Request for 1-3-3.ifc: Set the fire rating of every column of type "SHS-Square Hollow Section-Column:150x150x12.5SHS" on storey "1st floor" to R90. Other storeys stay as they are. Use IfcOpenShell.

First a look at what the model holds.

```python
import ifcopenshell
import ifcopenshell.util.element

model = ifcopenshell.open("1-3-3.ifc")
print(model.schema)
storey = next(s for s in model.by_type("IfcBuildingStorey") if s.Name == "1st floor")
columns = [e for e in ifcopenshell.util.element.get_decomposition(storey) if e.is_a("IfcColumn")]
seen = {}
for e in columns:
    element_type = ifcopenshell.util.element.get_type(e)
    key = (element_type.Name if element_type != e and element_type else None, ifcopenshell.util.element.get_pset(e, "Pset_ColumnCommon", "FireRating"))
    seen[key] = seen.get(key, 0) + 1
for (name, value), count in sorted(seen.items(), key=str):
    print(count, "x", name, "|", value)
```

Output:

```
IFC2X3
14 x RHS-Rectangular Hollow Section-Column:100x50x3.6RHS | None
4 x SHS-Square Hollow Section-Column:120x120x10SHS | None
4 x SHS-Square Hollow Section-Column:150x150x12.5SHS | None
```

```python
import ifcopenshell
import ifcopenshell.api.pset
import ifcopenshell.util.element

model = ifcopenshell.open("1-3-3.ifc")

storey = next(s for s in model.by_type("IfcBuildingStorey") if s.Name == "1st floor")
columns = [e for e in ifcopenshell.util.element.get_decomposition(storey) if e.is_a("IfcColumn")]

count = 0
for e in columns:
    element_type = ifcopenshell.util.element.get_type(e)
    if element_type in (None, e) or element_type.Name != "SHS-Square Hollow Section-Column:150x150x12.5SHS":
        continue
    # add_pset returns the element's existing set when there is one.
    pset = ifcopenshell.api.pset.add_pset(model, product=e, name="Pset_ColumnCommon")
    ifcopenshell.api.pset.edit_pset(model, pset=pset, properties={"FireRating": "R90"})
    count += 1

print(count, "columns updated")

model.write("1-3-3_updated.ifc")
```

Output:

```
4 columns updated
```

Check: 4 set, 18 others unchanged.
